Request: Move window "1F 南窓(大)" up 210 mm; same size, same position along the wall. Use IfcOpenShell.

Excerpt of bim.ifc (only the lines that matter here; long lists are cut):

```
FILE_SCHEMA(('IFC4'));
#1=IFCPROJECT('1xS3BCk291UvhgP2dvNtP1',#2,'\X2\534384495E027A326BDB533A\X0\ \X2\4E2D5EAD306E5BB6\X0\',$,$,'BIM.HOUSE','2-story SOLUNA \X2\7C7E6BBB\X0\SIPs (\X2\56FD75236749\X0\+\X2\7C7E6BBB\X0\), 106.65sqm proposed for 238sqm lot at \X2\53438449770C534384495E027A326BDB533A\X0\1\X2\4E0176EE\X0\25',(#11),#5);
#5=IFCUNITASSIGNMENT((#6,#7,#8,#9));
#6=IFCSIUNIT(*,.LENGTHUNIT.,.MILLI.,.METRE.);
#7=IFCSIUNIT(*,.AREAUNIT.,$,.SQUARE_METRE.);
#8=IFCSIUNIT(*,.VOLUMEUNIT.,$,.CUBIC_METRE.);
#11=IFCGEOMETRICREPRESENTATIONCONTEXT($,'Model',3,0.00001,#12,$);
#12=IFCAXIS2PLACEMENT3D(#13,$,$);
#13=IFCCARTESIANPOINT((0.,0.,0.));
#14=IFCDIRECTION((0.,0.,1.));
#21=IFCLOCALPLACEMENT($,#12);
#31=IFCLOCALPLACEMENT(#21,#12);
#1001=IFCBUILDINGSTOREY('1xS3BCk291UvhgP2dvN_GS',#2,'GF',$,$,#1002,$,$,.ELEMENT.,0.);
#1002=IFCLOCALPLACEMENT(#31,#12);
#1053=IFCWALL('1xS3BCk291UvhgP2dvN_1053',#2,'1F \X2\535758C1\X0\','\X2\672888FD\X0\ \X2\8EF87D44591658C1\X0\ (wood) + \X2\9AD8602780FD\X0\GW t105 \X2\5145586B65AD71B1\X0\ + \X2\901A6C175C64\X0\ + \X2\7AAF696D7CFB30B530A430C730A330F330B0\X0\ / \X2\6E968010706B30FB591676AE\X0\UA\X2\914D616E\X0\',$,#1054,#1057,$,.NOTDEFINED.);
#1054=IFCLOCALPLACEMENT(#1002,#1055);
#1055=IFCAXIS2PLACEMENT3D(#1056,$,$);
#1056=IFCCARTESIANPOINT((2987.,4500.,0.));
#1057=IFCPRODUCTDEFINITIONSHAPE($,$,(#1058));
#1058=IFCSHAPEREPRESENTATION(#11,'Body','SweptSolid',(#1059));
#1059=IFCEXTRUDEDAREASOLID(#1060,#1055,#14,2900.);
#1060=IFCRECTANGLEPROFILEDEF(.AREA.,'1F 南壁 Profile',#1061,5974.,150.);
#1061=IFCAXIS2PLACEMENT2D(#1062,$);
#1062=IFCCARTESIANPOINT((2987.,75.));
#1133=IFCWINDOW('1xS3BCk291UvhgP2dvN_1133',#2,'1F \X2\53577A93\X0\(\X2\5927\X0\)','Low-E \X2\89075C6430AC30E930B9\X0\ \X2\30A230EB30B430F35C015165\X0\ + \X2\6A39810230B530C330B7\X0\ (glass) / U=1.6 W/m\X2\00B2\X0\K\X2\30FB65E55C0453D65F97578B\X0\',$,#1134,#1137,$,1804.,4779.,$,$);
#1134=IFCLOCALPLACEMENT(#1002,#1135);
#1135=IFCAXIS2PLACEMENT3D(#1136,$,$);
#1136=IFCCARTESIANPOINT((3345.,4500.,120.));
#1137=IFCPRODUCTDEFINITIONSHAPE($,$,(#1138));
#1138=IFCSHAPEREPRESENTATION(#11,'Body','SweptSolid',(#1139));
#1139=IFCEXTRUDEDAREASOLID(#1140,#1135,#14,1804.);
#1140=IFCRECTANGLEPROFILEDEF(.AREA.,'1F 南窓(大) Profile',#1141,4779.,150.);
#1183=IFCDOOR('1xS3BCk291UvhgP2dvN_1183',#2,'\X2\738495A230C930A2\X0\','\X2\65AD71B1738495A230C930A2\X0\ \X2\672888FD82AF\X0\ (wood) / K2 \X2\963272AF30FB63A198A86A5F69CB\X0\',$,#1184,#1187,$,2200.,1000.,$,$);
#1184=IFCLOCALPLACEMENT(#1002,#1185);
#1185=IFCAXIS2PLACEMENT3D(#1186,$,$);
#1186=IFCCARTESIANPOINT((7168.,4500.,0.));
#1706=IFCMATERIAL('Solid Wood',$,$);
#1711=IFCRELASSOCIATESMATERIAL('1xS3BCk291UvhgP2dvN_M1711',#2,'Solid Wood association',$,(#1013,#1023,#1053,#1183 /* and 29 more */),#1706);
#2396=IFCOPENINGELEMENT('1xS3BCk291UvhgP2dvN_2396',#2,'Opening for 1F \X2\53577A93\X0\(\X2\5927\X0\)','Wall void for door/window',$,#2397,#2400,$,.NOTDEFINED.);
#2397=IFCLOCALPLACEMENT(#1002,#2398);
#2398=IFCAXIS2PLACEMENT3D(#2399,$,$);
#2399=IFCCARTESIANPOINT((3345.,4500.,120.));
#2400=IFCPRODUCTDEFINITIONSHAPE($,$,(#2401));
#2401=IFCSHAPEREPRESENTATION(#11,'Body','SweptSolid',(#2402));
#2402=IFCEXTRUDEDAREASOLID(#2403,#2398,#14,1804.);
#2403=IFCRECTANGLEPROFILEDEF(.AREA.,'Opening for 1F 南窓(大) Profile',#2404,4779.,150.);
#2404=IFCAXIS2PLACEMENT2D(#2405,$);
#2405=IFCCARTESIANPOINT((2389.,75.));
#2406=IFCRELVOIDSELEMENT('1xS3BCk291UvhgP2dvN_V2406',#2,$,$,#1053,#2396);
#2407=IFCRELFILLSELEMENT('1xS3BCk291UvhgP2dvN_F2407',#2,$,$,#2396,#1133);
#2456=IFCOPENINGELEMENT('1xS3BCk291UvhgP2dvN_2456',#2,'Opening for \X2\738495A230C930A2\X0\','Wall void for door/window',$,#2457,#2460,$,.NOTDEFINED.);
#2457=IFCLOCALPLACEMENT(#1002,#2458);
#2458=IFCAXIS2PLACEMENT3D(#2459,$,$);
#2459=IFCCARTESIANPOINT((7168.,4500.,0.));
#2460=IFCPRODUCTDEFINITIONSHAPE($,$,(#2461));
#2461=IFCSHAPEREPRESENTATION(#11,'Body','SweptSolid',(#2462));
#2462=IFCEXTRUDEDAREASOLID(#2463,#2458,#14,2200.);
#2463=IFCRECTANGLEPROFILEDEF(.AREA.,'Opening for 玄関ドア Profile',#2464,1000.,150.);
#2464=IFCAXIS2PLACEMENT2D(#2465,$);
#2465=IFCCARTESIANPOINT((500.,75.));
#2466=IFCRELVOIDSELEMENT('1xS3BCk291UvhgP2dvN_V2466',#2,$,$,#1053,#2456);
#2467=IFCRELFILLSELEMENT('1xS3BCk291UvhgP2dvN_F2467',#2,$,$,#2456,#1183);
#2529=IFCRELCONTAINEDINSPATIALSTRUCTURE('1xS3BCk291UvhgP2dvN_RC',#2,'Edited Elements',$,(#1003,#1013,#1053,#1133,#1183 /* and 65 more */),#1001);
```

```python
import numpy as np
import ifcopenshell
import ifcopenshell.api.geometry
import ifcopenshell.util.placement
import ifcopenshell.util.unit

model = ifcopenshell.open("bim.ifc")
unit_scale = ifcopenshell.util.unit.calculate_unit_scale(model)

window = model.by_guid("1xS3BCk291UvhgP2dvN_1133")
opening = window.FillsVoids[0].RelatingOpeningElement
dz = 210.0

shift = np.array([0.0, 0.0, dz])
# The window is not placed relative to its opening, so move both.
for product in (opening, window):
    matrix = ifcopenshell.util.placement.get_local_placement(product.ObjectPlacement)
    matrix[:3, 3] += shift
    ifcopenshell.api.geometry.edit_object_placement(model, product=product, matrix=matrix, is_si=False)

print(f"moved by {dz * unit_scale:+.3f} m")

model.write("bim_rev.ifc")
```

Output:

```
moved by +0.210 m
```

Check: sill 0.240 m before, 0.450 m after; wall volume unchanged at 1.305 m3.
